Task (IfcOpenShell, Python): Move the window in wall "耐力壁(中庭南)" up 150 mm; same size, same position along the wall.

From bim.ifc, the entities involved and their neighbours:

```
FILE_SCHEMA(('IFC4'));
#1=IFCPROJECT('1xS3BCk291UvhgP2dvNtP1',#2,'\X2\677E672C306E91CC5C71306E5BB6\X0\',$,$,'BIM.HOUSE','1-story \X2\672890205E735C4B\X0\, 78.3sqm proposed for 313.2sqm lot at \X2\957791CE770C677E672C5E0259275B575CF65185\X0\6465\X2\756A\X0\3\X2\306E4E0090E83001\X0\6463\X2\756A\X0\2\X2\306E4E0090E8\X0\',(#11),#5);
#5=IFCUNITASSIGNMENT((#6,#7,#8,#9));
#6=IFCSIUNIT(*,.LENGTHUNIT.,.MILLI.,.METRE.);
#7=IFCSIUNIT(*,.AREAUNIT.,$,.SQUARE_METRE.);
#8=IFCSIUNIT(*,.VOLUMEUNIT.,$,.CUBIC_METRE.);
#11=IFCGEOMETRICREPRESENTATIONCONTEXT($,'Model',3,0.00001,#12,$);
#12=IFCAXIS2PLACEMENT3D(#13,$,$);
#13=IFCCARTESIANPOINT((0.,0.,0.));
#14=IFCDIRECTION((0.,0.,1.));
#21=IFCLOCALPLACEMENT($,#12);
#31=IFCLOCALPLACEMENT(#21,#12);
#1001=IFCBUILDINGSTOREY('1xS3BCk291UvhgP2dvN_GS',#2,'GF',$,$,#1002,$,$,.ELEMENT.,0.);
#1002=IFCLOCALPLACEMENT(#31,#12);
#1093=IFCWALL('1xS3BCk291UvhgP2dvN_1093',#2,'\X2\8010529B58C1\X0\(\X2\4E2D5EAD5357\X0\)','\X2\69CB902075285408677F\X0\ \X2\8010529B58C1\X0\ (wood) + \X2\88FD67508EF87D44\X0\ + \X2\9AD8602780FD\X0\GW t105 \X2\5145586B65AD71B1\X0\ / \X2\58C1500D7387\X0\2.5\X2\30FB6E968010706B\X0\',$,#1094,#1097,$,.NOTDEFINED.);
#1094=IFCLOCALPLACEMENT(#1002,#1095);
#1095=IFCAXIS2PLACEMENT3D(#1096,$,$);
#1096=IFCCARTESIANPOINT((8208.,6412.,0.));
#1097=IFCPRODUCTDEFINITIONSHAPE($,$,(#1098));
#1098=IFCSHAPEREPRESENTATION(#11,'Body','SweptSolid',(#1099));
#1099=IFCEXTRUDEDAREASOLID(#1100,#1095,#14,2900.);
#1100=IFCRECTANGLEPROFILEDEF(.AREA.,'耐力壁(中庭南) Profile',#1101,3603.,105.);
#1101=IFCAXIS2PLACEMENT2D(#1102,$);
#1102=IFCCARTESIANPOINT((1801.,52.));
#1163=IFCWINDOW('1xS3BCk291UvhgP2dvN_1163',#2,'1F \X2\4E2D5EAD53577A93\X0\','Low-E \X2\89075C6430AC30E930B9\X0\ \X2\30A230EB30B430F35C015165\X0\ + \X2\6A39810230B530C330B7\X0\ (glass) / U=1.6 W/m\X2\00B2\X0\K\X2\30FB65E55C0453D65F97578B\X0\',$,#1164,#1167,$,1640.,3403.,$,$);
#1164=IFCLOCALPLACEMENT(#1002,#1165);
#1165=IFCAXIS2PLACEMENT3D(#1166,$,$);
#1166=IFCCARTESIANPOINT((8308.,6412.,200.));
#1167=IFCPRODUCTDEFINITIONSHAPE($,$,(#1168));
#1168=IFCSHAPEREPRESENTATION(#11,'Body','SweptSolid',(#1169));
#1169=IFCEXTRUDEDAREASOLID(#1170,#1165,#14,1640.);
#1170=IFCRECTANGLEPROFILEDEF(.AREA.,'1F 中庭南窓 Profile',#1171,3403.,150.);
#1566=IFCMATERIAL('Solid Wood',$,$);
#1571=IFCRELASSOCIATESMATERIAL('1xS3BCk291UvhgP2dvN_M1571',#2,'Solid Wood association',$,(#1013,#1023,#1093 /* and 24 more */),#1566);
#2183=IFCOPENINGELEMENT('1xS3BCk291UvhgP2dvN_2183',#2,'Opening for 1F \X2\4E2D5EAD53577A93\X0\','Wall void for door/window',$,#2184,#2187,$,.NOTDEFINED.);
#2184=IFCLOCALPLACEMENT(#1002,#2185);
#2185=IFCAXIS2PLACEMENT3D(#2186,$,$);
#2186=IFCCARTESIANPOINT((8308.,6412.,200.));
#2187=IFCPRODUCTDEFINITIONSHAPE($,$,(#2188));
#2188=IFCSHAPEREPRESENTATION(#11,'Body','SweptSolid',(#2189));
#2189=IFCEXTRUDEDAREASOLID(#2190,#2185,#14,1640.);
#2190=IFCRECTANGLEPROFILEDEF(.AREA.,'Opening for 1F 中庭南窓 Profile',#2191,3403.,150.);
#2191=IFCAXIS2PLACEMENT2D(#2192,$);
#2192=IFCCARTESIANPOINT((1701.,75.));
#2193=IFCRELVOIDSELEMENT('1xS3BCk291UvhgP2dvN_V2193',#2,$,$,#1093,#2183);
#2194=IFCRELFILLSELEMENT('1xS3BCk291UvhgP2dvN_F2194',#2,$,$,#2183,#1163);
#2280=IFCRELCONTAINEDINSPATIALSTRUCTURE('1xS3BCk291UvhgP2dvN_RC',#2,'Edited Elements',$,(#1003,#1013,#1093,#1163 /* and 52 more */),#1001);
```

```python
import numpy as np
import ifcopenshell
import ifcopenshell.api.geometry
import ifcopenshell.util.placement
import ifcopenshell.util.unit

model = ifcopenshell.open("bim.ifc")
unit_scale = ifcopenshell.util.unit.calculate_unit_scale(model)

window = model.by_guid("1xS3BCk291UvhgP2dvN_1163")
opening = window.FillsVoids[0].RelatingOpeningElement
dz = 0.15 / unit_scale

shift = np.array([0.0, 0.0, dz])
# The window is not placed relative to its opening, so move both.
for product in (opening, window):
    matrix = ifcopenshell.util.placement.get_local_placement(product.ObjectPlacement)
    matrix[:3, 3] += shift
    ifcopenshell.api.geometry.edit_object_placement(model, product=product, matrix=matrix, is_si=False)

print(f"moved by {dz * unit_scale:+.3f} m")

model.write("bim_updated.ifc")
```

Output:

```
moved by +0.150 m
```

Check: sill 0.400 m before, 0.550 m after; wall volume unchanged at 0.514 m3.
